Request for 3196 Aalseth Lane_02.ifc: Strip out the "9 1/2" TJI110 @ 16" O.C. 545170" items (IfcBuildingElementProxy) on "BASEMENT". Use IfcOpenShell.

First a look at what the model holds.

```python
import ifcopenshell
import ifcopenshell.util.element

model = ifcopenshell.open("3196 Aalseth Lane_02.ifc")
print(model.schema)
storey = next(s for s in model.by_type("IfcBuildingStorey") if s.Name == "BASEMENT")
proxies = [e for e in ifcopenshell.util.element.get_decomposition(storey) if e.is_a("IfcBuildingElementProxy")]
seen = {}
for e in proxies:
    element_type = ifcopenshell.util.element.get_type(e)
    name = element_type.Name if element_type not in (None, e) else None
    seen[name] = seen.get(name, 0) + 1
for name, count in sorted(seen.items(), key=str):
    print(count, "x", name)
```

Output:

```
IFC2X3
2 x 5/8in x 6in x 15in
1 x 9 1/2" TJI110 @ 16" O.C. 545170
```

```python
import ifcopenshell
import ifcopenshell.api.root
import ifcopenshell.util.element

model = ifcopenshell.open("3196 Aalseth Lane_02.ifc")

storey = next(s for s in model.by_type("IfcBuildingStorey") if s.Name == "BASEMENT")
proxies = [e for e in ifcopenshell.util.element.get_decomposition(storey) if e.is_a("IfcBuildingElementProxy")]
targets = [e for e in proxies if (t := ifcopenshell.util.element.get_type(e)) not in (None, e) and t.Name == '9 1/2" TJI110 @ 16" O.C. 545170']

for e in targets:
    ifcopenshell.api.root.remove_product(model, product=e)
print(len(targets), "removed")

model.write("3196 Aalseth Lane_02-out.ifc")
```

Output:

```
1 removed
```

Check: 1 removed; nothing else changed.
